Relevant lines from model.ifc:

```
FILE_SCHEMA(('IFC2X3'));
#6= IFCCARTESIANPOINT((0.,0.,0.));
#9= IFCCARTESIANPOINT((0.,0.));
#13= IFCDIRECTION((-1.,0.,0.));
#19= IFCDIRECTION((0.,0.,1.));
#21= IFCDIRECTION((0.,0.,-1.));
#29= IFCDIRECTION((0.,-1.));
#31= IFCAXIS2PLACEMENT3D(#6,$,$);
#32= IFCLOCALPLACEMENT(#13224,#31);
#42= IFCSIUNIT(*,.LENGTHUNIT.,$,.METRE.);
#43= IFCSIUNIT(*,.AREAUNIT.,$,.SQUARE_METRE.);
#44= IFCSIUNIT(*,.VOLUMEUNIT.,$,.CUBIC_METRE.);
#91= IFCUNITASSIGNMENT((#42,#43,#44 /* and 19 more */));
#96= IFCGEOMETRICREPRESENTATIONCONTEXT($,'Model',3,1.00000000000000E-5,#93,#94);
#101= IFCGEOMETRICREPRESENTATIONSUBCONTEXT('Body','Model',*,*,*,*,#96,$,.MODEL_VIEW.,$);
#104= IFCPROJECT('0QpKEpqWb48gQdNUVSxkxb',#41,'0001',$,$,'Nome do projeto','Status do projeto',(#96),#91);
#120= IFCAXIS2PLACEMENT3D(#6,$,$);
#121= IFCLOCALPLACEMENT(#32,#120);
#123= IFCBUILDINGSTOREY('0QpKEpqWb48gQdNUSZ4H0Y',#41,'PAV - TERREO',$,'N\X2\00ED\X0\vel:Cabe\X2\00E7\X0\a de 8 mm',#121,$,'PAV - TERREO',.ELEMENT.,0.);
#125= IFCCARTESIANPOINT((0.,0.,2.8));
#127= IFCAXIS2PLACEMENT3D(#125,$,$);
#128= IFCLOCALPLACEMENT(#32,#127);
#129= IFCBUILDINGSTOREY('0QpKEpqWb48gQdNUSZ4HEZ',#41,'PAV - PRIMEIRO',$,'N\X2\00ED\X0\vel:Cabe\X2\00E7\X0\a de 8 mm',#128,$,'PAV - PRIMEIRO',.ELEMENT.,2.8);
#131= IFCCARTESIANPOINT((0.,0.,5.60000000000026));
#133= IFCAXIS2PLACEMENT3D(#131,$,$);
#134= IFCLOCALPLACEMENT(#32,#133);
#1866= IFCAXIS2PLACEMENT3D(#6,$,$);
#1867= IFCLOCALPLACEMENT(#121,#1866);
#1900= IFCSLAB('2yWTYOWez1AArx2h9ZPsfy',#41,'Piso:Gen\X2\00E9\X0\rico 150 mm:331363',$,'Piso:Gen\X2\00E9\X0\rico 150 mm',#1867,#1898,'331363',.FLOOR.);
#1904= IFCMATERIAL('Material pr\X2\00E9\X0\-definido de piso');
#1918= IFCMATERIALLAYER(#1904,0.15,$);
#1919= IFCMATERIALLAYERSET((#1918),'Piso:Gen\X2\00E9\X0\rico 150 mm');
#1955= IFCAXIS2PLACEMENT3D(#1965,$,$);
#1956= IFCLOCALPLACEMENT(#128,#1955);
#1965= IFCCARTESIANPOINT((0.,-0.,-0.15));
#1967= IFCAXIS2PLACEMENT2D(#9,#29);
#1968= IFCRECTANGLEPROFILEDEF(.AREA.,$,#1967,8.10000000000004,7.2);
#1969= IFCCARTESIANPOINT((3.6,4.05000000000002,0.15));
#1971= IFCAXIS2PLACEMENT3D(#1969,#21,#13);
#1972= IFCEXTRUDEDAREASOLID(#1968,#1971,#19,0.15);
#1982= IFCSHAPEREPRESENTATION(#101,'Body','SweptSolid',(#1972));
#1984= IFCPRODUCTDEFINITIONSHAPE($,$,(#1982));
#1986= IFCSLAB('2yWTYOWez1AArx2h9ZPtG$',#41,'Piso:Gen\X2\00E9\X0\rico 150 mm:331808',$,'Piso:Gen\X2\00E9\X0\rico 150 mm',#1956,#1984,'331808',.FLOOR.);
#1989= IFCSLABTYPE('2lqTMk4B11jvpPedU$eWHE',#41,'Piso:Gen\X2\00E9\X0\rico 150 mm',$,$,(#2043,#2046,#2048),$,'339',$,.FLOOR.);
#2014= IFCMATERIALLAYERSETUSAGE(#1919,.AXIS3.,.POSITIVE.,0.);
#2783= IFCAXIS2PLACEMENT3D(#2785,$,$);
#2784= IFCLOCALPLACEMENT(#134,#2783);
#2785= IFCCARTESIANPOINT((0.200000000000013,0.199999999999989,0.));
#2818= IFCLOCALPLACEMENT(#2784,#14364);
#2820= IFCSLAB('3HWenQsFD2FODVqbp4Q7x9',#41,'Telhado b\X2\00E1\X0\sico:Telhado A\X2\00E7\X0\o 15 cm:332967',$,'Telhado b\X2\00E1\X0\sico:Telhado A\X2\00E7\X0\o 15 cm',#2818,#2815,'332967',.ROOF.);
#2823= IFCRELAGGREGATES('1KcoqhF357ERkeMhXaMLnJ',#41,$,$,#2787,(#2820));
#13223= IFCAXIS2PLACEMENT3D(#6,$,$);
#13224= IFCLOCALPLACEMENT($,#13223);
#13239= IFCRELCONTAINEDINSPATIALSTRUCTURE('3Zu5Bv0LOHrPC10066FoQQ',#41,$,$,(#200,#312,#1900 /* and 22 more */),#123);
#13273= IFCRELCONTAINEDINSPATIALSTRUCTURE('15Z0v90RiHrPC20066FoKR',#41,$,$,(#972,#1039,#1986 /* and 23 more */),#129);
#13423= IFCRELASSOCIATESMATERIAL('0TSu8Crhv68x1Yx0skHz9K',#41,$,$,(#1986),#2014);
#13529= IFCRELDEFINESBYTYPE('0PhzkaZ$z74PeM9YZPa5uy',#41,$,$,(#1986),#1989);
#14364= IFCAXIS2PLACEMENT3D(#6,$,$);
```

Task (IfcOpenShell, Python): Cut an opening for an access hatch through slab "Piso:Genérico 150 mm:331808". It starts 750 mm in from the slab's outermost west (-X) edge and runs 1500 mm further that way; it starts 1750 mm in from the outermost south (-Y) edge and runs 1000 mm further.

```python
import numpy as np
import ifcopenshell
import ifcopenshell.api.feature
import ifcopenshell.api.geometry
import ifcopenshell.api.root
import ifcopenshell.geom
import ifcopenshell.util.placement
import ifcopenshell.util.representation
import ifcopenshell.util.shape
import ifcopenshell.util.unit

model = ifcopenshell.open("model.ifc")
unit_scale = ifcopenshell.util.unit.calculate_unit_scale(model)
settings = ifcopenshell.geom.settings()


def volume(element):
    """Net volume in cubic metres, openings subtracted."""
    shape = ifcopenshell.geom.create_shape(settings, element)
    return ifcopenshell.util.shape.get_volume(shape.geometry)


slab = model.by_guid("2yWTYOWez1AArx2h9ZPtG$")
before = volume(slab)

# Extent in the slab's own axes, in metres. The edges named are its -X and -Y sides.
slab_shape = ifcopenshell.geom.create_shape(settings, slab)
vertices = ifcopenshell.util.shape.get_vertices(slab_shape.geometry)
x_min, y_min, bottom = vertices.min(axis=0)
top = vertices[:, 2].max()

opening = ifcopenshell.api.root.create_entity(model, ifc_class="IfcOpeningElement", name="Access hatch opening")
context = ifcopenshell.util.representation.get_context(model, "Model", "Body", "MODEL_VIEW")
width, depth = 1.5, 1
outline = [(0.0, 0.0), (width, 0.0), (width, depth), (0.0, depth), (0.0, 0.0)]
# Overshoot both faces by 50 mm so the cut is clean.
shape = ifcopenshell.api.geometry.add_slab_representation(
    model, context=context, depth=top - bottom + 0.1, polyline=outline
)
ifcopenshell.api.geometry.assign_representation(model, product=opening, representation=shape)

matrix = ifcopenshell.util.placement.get_local_placement(slab.ObjectPlacement)
matrix[:, 3] = matrix @ np.append(np.array([x_min + 0.75, y_min + 1.75, bottom - 0.05]) / unit_scale, 1.0)
ifcopenshell.api.geometry.edit_object_placement(model, product=opening, matrix=matrix, is_si=False)
ifcopenshell.api.feature.add_feature(model, feature=opening, element=slab)

after = volume(slab)

print(f"slab volume {before:.3f} -> {after:.3f} m3")

model.write("model_v2.ifc")
```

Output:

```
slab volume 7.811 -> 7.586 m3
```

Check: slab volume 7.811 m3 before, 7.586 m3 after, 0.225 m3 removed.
